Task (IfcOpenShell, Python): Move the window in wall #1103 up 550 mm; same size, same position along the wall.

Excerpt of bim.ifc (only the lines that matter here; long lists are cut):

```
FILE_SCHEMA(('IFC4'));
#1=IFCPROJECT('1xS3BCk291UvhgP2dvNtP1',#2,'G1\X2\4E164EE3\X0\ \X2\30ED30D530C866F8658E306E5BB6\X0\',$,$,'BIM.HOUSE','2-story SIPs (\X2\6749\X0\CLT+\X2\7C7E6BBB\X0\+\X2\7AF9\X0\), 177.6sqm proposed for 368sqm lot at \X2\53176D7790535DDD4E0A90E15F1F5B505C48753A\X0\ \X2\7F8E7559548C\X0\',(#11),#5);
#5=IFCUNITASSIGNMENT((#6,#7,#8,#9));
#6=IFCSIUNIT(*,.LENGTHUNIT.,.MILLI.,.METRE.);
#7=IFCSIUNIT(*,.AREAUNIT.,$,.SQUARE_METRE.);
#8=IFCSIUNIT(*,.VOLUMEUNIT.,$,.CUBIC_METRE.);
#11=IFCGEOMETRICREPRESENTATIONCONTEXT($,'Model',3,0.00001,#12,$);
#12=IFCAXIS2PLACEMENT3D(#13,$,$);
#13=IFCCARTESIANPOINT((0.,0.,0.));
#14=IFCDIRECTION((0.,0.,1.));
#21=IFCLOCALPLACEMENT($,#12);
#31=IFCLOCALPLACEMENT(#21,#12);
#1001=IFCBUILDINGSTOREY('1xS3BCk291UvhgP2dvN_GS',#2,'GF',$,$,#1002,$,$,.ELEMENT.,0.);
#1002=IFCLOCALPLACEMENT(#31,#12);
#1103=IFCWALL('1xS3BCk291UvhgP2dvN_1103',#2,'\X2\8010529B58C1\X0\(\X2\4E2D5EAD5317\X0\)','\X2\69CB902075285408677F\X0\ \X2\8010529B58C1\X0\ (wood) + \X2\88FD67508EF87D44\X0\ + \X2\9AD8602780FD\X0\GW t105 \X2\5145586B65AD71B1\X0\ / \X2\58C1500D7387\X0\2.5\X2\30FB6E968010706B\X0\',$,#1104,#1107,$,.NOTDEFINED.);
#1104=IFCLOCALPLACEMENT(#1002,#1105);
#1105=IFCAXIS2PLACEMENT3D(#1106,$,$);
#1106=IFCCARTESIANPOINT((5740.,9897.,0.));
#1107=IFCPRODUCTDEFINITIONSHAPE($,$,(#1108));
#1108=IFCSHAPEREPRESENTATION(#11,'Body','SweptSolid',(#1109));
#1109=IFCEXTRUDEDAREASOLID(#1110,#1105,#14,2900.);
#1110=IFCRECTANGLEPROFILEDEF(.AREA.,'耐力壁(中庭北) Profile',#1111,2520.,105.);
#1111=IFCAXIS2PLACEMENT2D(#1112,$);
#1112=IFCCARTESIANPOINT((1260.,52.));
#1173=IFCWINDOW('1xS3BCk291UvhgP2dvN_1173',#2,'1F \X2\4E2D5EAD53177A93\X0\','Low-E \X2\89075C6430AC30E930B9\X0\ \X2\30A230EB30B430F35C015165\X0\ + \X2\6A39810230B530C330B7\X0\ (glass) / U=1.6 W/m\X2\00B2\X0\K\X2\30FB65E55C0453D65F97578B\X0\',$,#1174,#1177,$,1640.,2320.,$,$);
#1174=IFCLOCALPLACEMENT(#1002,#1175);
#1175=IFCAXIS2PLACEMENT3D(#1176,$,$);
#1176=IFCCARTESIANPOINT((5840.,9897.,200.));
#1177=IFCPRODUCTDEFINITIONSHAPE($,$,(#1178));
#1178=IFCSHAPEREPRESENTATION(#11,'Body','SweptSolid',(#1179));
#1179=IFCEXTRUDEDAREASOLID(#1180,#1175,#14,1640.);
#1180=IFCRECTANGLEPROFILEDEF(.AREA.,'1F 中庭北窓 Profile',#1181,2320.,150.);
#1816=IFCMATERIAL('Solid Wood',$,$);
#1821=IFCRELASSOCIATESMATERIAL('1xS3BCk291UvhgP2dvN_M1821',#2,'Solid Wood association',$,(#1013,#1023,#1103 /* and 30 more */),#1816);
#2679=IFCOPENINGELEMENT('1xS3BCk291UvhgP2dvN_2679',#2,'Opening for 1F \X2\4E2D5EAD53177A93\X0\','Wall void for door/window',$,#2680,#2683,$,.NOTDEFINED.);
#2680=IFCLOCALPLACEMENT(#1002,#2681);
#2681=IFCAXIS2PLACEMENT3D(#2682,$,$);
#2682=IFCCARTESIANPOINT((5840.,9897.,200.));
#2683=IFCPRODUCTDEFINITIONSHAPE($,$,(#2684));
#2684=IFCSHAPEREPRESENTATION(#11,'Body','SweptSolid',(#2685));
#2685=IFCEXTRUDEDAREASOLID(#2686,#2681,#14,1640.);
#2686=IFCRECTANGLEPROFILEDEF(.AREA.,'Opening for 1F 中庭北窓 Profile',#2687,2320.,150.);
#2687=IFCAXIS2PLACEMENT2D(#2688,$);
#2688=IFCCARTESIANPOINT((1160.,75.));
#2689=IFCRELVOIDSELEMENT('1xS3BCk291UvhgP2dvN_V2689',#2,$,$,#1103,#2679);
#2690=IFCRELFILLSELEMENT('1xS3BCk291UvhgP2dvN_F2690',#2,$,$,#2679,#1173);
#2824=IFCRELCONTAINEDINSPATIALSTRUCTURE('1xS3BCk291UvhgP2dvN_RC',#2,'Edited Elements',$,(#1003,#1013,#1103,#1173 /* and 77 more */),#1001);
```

```python
import numpy as np
import ifcopenshell
import ifcopenshell.api.geometry
import ifcopenshell.util.placement
import ifcopenshell.util.unit

model = ifcopenshell.open("bim.ifc")
unit_scale = ifcopenshell.util.unit.calculate_unit_scale(model)

window = model.by_guid("1xS3BCk291UvhgP2dvN_1173")
opening = window.FillsVoids[0].RelatingOpeningElement
dz = 550.0

shift = np.array([0.0, 0.0, dz])
# The window is not placed relative to its opening, so move both.
for product in (opening, window):
    matrix = ifcopenshell.util.placement.get_local_placement(product.ObjectPlacement)
    matrix[:3, 3] += shift
    ifcopenshell.api.geometry.edit_object_placement(model, product=product, matrix=matrix, is_si=False)

print(f"moved by {dz * unit_scale:+.3f} m")

model.write("bim_v2.ifc")
```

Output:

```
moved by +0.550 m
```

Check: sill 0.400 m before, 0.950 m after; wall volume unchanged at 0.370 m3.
